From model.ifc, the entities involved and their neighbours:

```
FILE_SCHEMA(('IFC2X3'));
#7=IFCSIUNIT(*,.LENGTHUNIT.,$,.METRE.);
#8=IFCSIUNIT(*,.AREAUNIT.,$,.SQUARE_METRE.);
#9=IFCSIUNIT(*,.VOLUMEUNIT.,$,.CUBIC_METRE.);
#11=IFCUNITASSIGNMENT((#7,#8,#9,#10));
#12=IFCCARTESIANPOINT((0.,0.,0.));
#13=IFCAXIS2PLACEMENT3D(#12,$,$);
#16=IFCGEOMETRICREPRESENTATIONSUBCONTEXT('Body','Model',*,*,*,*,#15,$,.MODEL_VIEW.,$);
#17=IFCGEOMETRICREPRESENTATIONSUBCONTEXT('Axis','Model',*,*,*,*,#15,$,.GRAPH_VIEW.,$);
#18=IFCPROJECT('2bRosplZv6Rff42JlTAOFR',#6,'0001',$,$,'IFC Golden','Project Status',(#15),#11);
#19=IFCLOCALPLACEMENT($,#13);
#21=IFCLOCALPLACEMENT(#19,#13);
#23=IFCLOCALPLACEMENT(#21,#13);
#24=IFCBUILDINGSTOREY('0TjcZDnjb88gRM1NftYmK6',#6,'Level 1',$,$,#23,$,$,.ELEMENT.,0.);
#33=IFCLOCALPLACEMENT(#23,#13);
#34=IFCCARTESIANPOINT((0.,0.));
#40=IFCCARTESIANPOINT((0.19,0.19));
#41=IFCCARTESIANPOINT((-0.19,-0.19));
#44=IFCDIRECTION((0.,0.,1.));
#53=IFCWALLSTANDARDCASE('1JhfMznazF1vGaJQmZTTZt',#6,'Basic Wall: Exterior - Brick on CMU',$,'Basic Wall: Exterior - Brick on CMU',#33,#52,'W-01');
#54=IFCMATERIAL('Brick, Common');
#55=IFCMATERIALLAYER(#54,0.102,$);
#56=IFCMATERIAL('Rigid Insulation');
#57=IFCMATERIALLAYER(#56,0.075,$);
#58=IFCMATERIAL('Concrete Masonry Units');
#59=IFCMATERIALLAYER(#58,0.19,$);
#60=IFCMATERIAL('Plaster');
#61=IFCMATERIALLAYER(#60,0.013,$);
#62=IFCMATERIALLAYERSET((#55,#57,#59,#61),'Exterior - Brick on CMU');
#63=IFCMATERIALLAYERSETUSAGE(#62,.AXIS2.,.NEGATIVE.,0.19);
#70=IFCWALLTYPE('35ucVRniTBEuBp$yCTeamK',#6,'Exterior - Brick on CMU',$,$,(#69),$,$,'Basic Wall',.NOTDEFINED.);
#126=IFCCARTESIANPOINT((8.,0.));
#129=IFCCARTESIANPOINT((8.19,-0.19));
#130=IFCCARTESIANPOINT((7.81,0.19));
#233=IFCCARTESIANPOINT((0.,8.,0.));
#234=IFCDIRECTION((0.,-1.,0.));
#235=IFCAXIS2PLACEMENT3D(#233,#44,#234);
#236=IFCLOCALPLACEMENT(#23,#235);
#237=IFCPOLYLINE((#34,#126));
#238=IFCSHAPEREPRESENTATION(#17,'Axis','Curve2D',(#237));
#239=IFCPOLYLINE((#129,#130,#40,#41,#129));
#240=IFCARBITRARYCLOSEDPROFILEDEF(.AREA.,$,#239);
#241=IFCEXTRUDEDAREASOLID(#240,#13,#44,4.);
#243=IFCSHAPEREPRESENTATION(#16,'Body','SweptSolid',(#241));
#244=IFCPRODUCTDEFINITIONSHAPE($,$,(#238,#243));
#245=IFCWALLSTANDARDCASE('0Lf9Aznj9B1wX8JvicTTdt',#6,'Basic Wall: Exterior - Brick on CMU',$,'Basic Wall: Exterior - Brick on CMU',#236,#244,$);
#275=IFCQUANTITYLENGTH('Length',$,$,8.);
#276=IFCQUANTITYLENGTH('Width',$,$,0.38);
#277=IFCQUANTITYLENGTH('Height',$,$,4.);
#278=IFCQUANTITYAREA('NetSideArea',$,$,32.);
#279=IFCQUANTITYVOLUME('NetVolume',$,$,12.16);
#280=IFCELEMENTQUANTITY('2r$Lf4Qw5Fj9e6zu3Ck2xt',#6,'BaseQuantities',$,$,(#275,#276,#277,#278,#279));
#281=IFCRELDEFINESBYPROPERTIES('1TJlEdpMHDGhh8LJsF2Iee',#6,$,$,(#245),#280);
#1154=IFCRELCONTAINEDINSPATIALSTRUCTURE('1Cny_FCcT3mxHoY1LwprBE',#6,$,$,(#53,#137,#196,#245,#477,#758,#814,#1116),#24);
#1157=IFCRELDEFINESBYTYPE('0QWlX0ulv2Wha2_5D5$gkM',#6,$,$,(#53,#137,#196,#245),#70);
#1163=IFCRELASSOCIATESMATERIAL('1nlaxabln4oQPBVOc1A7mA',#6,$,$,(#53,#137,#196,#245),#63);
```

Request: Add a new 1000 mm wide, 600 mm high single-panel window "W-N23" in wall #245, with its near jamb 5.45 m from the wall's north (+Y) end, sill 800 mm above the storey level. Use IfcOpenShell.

```python
import numpy as np
import ifcopenshell
import ifcopenshell.api.feature
import ifcopenshell.api.geometry
import ifcopenshell.api.pset
import ifcopenshell.api.root
import ifcopenshell.api.spatial
import ifcopenshell.api.type
import ifcopenshell.geom
import ifcopenshell.util.element
import ifcopenshell.util.placement
import ifcopenshell.util.representation
import ifcopenshell.util.shape
import ifcopenshell.util.unit

model = ifcopenshell.open("model.ifc")
unit_scale = ifcopenshell.util.unit.calculate_unit_scale(model)
area_scale = ifcopenshell.util.unit.calculate_unit_scale(model, "AREAUNIT")
volume_scale = ifcopenshell.util.unit.calculate_unit_scale(model, "VOLUMEUNIT")
settings = ifcopenshell.geom.settings()


def volume(element):
    """Net volume in cubic metres, openings subtracted."""
    shape = ifcopenshell.geom.create_shape(settings, element)
    return ifcopenshell.util.shape.get_volume(shape.geometry)


wall = model.by_guid("0Lf9Aznj9B1wX8JvicTTdt")
storey = ifcopenshell.util.element.get_container(wall, ifc_class="IfcBuildingStorey")
context = ifcopenshell.util.representation.get_context(model, "Model", "Body", "MODEL_VIEW")
before = volume(wall)

width, height, from_end, sill = 1, 0.6, 5.45, 0.8  # metres

# The wall runs along its own X axis, and the end named is its -X end.
wall_shape = ifcopenshell.geom.create_shape(settings, wall)
x, y, z = ifcopenshell.util.shape.get_vertices(wall_shape.geometry).T
start = x.min() + from_end
face, thickness = float(y.min()), float(y.max() - y.min())
wall_matrix = ifcopenshell.util.placement.get_local_placement(wall.ObjectPlacement)
level = ifcopenshell.util.placement.get_local_placement(storey.ObjectPlacement)[2, 3]


def in_wall(x, y):
    """Placement at x, y metres in the wall's axes, at sill height."""
    matrix = wall_matrix.copy()
    matrix[:, 3] = wall_matrix @ np.array([x / unit_scale, y / unit_scale, 0.0, 1.0])
    matrix[2, 3] = level + sill / unit_scale
    return matrix


# Opening: a box that overshoots both wall faces by 50 mm.
opening = ifcopenshell.api.root.create_entity(model, ifc_class="IfcOpeningElement")
box = ifcopenshell.api.geometry.add_wall_representation(
    model, context=context, length=width, height=height, thickness=thickness + 0.1
)
ifcopenshell.api.geometry.assign_representation(model, product=opening, representation=box)
ifcopenshell.api.geometry.edit_object_placement(model, product=opening, matrix=in_wall(start, face - 0.05), is_si=False)
ifcopenshell.api.feature.add_feature(model, feature=opening, element=wall)

window = ifcopenshell.api.root.create_entity(model, ifc_class="IfcWindow", name="W-N23")
window.OverallWidth, window.OverallHeight = width / unit_scale, height / unit_scale
body = ifcopenshell.api.geometry.add_window_representation(
    model,
    context=context,
    overall_width=window.OverallWidth,
    overall_height=window.OverallHeight,
    partition_type="SINGLE_PANEL",
)
ifcopenshell.api.geometry.assign_representation(model, product=window, representation=body)
ifcopenshell.api.spatial.assign_container(model, products=[window], relating_structure=storey)
fills = ifcopenshell.api.feature.add_filling(model, opening=opening, element=window)
fills.OwnerHistory = window.OwnerHistory  # required in IFC2X3

# IFC2X3 keeps the operation on the window style.
style = ifcopenshell.api.root.create_entity(model, ifc_class="IfcWindowStyle", name="W-N23")
style.OperationType, style.ConstructionType = "SINGLE_PANEL", "NOTDEFINED"
style.ParameterTakesPrecedence = style.Sizeable = False
ifcopenshell.api.type.assign_type(model, related_objects=[window], relating_type=style)

# Centre the window in the wall's thickness.
ifcopenshell.api.geometry.edit_object_placement(model, product=window, matrix=in_wall(start, face), is_si=False)
window_shape = ifcopenshell.geom.create_shape(settings, window)
depth = ifcopenshell.util.shape.get_vertices(window_shape.geometry)[:, 1]
offset = face + thickness / 2 - (depth.min() + depth.max()) / 2
ifcopenshell.api.geometry.edit_object_placement(model, product=window, matrix=in_wall(start, offset), is_si=False)

after = volume(wall)

# Update the wall's stored quantities.
qto = model.by_id(ifcopenshell.util.element.get_pset(wall, "BaseQuantities", should_inherit=False)["id"])
ifcopenshell.api.pset.edit_qto(model, qto=qto, properties={
    "NetSideArea": after / thickness / area_scale,
    "NetVolume": after / volume_scale,
})

print(f"wall volume {before:.3f} -> {after:.3f} m3")

model.write("model_rev.ifc")
```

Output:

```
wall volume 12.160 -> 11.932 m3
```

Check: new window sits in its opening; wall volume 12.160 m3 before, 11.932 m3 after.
